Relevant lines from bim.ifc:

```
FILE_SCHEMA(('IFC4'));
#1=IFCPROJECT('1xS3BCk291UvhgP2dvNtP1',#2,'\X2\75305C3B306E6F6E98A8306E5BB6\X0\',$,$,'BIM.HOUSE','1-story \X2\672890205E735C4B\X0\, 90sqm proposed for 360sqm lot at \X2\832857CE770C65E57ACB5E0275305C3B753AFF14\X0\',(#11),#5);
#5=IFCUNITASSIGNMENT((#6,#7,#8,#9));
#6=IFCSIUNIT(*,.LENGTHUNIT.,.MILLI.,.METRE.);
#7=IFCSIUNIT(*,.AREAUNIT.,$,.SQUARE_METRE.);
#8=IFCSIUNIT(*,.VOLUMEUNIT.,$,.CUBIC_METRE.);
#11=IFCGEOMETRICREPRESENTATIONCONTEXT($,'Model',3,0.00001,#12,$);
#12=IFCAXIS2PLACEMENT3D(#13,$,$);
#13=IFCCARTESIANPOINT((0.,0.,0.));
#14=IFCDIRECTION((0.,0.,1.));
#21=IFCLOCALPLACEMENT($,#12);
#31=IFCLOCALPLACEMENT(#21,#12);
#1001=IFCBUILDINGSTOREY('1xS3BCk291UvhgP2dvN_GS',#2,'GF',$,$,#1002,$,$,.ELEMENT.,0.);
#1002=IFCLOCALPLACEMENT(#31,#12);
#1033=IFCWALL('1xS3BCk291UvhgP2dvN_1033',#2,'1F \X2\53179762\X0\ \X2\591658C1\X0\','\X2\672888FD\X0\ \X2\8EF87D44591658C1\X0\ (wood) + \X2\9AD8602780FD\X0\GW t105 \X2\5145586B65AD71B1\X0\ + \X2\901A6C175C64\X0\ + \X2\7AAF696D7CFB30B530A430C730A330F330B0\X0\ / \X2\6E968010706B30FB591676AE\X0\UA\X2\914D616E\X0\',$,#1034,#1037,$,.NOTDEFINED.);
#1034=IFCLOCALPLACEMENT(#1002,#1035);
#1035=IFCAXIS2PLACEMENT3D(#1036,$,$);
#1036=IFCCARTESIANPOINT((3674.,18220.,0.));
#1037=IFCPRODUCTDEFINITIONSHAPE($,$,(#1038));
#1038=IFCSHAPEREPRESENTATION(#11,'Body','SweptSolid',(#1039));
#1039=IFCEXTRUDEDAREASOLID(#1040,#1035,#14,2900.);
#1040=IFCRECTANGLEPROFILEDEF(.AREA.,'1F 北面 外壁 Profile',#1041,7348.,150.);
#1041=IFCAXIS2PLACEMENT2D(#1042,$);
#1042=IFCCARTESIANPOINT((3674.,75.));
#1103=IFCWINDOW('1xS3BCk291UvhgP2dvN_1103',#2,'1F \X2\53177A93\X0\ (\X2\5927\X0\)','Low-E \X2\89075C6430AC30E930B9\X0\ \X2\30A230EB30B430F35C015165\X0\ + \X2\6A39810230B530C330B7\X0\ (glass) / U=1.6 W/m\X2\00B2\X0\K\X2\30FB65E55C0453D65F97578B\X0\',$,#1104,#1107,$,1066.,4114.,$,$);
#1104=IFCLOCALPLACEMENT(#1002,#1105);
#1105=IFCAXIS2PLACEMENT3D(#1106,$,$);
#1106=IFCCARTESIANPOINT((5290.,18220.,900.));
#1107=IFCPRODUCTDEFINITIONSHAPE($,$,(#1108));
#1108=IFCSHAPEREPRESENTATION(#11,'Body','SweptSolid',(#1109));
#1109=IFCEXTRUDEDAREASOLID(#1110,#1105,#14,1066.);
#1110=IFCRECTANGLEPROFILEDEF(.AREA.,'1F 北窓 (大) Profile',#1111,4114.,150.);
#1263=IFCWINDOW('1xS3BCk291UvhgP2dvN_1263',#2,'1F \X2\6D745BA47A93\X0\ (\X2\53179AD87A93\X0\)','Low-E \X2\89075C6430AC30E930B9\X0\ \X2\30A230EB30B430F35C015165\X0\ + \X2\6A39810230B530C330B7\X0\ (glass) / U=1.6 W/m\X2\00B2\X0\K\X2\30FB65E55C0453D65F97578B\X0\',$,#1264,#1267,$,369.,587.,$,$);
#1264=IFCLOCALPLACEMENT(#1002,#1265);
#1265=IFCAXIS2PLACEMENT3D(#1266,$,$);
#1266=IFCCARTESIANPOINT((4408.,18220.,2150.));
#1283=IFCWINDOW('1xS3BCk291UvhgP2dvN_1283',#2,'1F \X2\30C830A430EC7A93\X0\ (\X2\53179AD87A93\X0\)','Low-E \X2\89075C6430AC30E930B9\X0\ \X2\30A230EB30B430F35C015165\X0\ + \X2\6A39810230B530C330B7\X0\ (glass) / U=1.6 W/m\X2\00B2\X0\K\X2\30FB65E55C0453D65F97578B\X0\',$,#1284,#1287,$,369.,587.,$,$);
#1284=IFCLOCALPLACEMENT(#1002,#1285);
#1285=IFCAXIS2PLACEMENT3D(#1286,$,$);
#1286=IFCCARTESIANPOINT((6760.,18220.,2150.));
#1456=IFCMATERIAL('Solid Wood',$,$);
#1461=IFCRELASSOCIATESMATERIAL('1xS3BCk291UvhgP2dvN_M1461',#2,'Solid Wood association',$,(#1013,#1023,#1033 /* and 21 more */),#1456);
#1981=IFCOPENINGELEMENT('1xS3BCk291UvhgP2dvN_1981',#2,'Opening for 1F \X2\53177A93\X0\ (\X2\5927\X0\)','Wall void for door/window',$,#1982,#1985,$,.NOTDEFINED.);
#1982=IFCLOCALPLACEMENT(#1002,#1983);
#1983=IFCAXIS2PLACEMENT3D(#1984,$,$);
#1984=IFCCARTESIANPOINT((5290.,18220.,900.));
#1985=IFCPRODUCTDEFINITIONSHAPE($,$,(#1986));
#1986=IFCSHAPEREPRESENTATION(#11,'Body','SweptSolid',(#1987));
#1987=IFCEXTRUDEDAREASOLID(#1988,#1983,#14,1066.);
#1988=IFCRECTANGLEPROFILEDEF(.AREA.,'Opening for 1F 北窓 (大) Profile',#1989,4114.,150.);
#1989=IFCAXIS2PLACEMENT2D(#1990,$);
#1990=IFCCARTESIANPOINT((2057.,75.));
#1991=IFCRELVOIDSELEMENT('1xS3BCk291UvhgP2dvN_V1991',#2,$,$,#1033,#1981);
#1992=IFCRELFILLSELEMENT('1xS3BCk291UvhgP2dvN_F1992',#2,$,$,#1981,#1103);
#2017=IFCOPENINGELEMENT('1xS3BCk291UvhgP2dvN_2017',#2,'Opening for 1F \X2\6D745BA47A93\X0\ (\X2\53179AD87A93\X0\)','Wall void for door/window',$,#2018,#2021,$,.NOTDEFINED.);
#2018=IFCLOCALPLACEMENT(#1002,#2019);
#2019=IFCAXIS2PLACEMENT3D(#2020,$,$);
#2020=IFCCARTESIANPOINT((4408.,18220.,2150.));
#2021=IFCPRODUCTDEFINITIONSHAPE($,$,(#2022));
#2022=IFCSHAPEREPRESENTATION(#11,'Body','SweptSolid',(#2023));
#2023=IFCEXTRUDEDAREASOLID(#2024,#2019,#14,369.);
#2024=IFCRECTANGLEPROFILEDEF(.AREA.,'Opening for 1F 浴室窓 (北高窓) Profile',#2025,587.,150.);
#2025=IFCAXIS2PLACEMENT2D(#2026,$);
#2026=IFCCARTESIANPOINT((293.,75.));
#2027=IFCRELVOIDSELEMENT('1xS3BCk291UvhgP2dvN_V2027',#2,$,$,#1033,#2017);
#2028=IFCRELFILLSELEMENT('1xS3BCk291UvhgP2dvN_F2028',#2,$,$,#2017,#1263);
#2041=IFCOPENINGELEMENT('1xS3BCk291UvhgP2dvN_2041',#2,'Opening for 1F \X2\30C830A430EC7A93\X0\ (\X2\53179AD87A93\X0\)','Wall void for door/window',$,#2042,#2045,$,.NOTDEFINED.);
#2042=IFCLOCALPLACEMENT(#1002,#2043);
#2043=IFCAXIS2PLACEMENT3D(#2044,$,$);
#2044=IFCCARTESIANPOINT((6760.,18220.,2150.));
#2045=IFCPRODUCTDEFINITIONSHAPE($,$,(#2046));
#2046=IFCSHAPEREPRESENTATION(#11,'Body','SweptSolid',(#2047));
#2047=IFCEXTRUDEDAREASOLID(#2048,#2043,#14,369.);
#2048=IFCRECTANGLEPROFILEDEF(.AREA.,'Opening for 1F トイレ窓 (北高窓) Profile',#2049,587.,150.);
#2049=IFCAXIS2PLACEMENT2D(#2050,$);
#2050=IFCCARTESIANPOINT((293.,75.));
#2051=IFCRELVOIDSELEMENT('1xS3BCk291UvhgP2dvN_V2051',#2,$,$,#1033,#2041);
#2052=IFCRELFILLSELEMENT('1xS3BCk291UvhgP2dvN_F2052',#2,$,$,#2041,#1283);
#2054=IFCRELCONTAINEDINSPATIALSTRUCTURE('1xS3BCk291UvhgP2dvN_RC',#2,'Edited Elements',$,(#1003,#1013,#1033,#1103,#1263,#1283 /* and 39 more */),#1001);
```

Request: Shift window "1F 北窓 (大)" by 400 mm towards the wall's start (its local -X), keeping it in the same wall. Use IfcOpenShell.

```python
import ifcopenshell
import ifcopenshell.api.geometry
import ifcopenshell.util.placement
import ifcopenshell.util.unit

model = ifcopenshell.open("bim.ifc")
unit_scale = ifcopenshell.util.unit.calculate_unit_scale(model)

window = model.by_guid("1xS3BCk291UvhgP2dvN_1103")
opening = window.FillsVoids[0].RelatingOpeningElement
wall = opening.VoidsElements[0].RelatingBuildingElement

wall_matrix = ifcopenshell.util.placement.get_local_placement(wall.ObjectPlacement)
shift = wall_matrix[:3, 0] * -0.4 / unit_scale
before = ifcopenshell.util.placement.get_local_placement(window.ObjectPlacement)[:3, 3].copy()

# The window is not placed relative to its opening, so move both.
for product in (opening, window):
    matrix = ifcopenshell.util.placement.get_local_placement(product.ObjectPlacement)
    matrix[:3, 3] += shift
    ifcopenshell.api.geometry.edit_object_placement(model, product=product, matrix=matrix, is_si=False)

after = ifcopenshell.util.placement.get_local_placement(window.ObjectPlacement)[:3, 3]
print("window moved by", (after - before).round(3) + 0.0)

model.write("bim_updated.ifc")
```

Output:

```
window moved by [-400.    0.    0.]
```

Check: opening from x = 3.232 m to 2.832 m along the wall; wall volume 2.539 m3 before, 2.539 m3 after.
